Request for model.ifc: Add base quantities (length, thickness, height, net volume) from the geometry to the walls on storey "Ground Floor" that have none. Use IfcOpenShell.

First a look at what the model holds.

```python
import ifcopenshell
import ifcopenshell.util.element
import ifcopenshell.util.unit

model = ifcopenshell.open("model.ifc")
print(model.schema)
for unit_type in ("LENGTHUNIT", "AREAUNIT", "VOLUMEUNIT"):
    print(unit_type, ifcopenshell.util.unit.calculate_unit_scale(model, unit_type))
storey = next(s for s in model.by_type("IfcBuildingStorey") if s.Name == "Ground Floor")
walls = [e for e in ifcopenshell.util.element.get_decomposition(storey) if e.is_a("IfcWall")]
for e in sorted(walls, key=lambda e: e.id()):
    print(e.id(), e.is_a(), e.Name, list(ifcopenshell.util.element.get_psets(e, qtos_only=True)), sep=" | ")
```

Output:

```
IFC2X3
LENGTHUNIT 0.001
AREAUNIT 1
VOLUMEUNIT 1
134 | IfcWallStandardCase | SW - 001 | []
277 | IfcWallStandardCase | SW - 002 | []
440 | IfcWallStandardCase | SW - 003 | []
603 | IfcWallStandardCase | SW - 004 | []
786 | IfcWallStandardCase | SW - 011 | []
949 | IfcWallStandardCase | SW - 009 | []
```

```python
import ifcopenshell
import ifcopenshell.api.pset
import ifcopenshell.geom
import ifcopenshell.util.element
import ifcopenshell.util.shape
import ifcopenshell.util.unit

model = ifcopenshell.open("model.ifc")
unit_scale = ifcopenshell.util.unit.calculate_unit_scale(model)
volume_scale = ifcopenshell.util.unit.calculate_unit_scale(model, "VOLUMEUNIT")
settings = ifcopenshell.geom.settings()

storey = next(s for s in model.by_type("IfcBuildingStorey") if s.Name == "Ground Floor")
walls = [e for e in ifcopenshell.util.element.get_decomposition(storey) if e.is_a("IfcWall")]

for e in sorted(walls, key=lambda e: e.id()):
    if ifcopenshell.util.element.get_psets(e, qtos_only=True, should_inherit=False):
        continue
    # Geometry comes back in metres, in the element's own axes.
    shape = ifcopenshell.geom.create_shape(settings, e)
    values = {
        "Length": ifcopenshell.util.shape.get_x(shape.geometry) / unit_scale,
        "Width": ifcopenshell.util.shape.get_y(shape.geometry) / unit_scale,
        "Height": ifcopenshell.util.shape.get_z(shape.geometry) / unit_scale,
        "NetVolume": ifcopenshell.util.shape.get_volume(shape.geometry) / volume_scale,
    }
    qto = ifcopenshell.api.pset.add_qto(model, product=e, name="BaseQuantities")
    ifcopenshell.api.pset.edit_qto(model, qto=qto, properties=values)
    print(e.id(), {k: round(v, 3) for k, v in values.items()})

model.write("model_rev.ifc")
```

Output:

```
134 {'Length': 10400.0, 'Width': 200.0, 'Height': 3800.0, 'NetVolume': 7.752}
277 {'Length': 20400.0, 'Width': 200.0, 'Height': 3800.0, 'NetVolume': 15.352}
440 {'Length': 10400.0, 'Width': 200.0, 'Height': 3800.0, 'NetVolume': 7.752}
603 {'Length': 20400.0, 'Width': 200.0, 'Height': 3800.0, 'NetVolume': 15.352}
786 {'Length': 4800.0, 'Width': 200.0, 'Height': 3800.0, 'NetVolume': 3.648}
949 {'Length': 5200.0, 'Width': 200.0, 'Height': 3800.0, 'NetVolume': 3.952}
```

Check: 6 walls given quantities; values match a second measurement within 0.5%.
